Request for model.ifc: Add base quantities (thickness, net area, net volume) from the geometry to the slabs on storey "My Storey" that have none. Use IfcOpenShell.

First a look at what the model holds.

```python
import ifcopenshell
import ifcopenshell.util.element
import ifcopenshell.util.unit

model = ifcopenshell.open("model.ifc")
print(model.schema)
for unit_type in ("LENGTHUNIT", "AREAUNIT", "VOLUMEUNIT"):
    print(unit_type, ifcopenshell.util.unit.calculate_unit_scale(model, unit_type))
storey = next(s for s in model.by_type("IfcBuildingStorey") if s.Name == "My Storey")
slabs = [e for e in ifcopenshell.util.element.get_decomposition(storey) if e.is_a("IfcSlab")]
for e in sorted(slabs, key=lambda e: e.id()):
    print(e.id(), e.is_a(), e.Name, list(ifcopenshell.util.element.get_psets(e, qtos_only=True)), sep=" | ")
```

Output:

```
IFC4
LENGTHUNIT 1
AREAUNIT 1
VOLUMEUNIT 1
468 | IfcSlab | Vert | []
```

```python
import ifcopenshell
import ifcopenshell.api.pset
import ifcopenshell.geom
import ifcopenshell.util.element
import ifcopenshell.util.shape
import ifcopenshell.util.unit

model = ifcopenshell.open("model.ifc")
unit_scale = ifcopenshell.util.unit.calculate_unit_scale(model)
area_scale = ifcopenshell.util.unit.calculate_unit_scale(model, "AREAUNIT")
volume_scale = ifcopenshell.util.unit.calculate_unit_scale(model, "VOLUMEUNIT")
settings = ifcopenshell.geom.settings()

storey = next(s for s in model.by_type("IfcBuildingStorey") if s.Name == "My Storey")
slabs = [e for e in ifcopenshell.util.element.get_decomposition(storey) if e.is_a("IfcSlab")]

for e in sorted(slabs, key=lambda e: e.id()):
    if ifcopenshell.util.element.get_psets(e, qtos_only=True, should_inherit=False):
        continue
    # Geometry comes back in metres, in the element's own axes.
    shape = ifcopenshell.geom.create_shape(settings, e)
    values = {
        "Width": ifcopenshell.util.shape.get_z(shape.geometry) / unit_scale,
        "NetArea": ifcopenshell.util.shape.get_footprint_area(shape.geometry) / area_scale,
        "NetVolume": ifcopenshell.util.shape.get_volume(shape.geometry) / volume_scale,
    }
    qto = ifcopenshell.api.pset.add_qto(model, product=e, name="Qto_SlabBaseQuantities")
    ifcopenshell.api.pset.edit_qto(model, qto=qto, properties=values)
    print(e.id(), {k: round(v, 3) for k, v in values.items()})

model.write("model_rev.ifc")
```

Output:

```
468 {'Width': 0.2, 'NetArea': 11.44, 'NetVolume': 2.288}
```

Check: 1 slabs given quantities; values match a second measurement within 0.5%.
